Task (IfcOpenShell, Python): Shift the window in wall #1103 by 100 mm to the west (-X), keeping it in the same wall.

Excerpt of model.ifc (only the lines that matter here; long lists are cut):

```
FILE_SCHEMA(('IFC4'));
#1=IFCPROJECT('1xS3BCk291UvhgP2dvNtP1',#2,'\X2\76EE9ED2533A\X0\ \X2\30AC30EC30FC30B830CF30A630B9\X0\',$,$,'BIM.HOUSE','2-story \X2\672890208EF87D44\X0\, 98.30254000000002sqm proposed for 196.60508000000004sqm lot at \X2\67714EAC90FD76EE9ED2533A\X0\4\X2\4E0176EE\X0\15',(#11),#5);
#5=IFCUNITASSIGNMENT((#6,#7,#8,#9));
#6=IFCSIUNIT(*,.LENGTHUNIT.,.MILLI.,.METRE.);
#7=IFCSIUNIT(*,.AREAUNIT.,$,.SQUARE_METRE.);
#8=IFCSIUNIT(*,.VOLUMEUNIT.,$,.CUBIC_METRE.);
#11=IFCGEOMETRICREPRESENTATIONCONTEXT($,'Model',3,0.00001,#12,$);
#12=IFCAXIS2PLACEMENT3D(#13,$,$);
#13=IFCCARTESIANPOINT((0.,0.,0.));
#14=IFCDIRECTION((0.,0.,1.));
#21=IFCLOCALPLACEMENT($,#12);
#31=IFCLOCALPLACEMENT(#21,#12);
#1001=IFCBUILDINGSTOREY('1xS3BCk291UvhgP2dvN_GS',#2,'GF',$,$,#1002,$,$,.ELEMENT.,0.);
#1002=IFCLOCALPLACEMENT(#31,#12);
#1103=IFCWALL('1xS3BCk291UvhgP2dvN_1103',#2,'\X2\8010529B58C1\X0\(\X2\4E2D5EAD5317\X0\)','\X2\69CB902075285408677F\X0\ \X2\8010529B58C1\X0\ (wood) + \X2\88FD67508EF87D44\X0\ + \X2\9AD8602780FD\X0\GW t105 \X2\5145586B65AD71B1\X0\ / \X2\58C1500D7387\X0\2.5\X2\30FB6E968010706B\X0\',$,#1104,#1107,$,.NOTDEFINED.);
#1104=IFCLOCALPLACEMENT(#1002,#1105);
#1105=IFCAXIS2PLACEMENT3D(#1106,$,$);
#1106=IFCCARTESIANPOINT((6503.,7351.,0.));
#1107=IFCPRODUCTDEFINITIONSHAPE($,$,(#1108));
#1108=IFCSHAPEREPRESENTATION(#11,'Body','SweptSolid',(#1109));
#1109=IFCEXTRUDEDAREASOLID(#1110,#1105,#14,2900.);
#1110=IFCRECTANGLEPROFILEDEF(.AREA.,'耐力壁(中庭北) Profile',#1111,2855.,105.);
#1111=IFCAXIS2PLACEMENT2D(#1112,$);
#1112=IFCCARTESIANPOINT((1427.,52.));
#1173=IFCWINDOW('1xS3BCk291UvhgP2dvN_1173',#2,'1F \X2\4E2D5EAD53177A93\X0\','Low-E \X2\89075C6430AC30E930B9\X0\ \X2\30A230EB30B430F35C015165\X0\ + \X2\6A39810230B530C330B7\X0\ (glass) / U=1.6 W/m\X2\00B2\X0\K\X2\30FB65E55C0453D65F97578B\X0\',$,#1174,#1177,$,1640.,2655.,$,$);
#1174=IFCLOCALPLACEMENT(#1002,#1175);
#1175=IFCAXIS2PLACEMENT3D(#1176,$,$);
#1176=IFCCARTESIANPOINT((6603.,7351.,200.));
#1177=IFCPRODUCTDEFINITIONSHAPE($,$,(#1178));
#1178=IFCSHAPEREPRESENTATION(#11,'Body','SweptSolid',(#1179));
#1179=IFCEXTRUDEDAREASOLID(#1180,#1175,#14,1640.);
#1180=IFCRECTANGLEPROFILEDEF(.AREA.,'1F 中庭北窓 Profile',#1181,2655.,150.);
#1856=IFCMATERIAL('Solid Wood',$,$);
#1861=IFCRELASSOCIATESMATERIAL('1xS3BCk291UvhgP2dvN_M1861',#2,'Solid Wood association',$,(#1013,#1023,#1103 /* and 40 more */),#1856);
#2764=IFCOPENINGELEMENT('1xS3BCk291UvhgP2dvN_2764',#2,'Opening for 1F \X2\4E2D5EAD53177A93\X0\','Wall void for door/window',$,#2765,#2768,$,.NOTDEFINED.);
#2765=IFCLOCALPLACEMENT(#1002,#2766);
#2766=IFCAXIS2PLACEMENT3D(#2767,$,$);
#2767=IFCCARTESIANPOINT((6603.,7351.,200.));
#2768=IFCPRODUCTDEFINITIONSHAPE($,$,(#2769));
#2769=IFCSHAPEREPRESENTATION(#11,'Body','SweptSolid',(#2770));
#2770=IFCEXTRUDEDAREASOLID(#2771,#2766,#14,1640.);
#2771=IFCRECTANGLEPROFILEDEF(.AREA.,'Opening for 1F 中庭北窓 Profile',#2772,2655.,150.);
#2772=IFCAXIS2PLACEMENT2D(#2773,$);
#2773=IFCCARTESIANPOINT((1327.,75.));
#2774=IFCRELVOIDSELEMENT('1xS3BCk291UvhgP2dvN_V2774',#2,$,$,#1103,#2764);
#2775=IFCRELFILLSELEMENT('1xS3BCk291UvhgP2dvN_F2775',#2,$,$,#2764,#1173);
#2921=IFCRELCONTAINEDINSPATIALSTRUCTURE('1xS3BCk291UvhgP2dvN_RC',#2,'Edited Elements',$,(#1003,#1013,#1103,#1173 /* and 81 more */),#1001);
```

```python
import ifcopenshell
import ifcopenshell.api.geometry
import ifcopenshell.util.placement

model = ifcopenshell.open("model.ifc")

window = model.by_guid("1xS3BCk291UvhgP2dvN_1173")
opening = window.FillsVoids[0].RelatingOpeningElement
wall = opening.VoidsElements[0].RelatingBuildingElement

wall_matrix = ifcopenshell.util.placement.get_local_placement(wall.ObjectPlacement)
shift = wall_matrix[:3, 0] * -100.0
before = ifcopenshell.util.placement.get_local_placement(window.ObjectPlacement)[:3, 3].copy()

# The window is not placed relative to its opening, so move both.
for product in (opening, window):
    matrix = ifcopenshell.util.placement.get_local_placement(product.ObjectPlacement)
    matrix[:3, 3] += shift
    ifcopenshell.api.geometry.edit_object_placement(model, product=product, matrix=matrix, is_si=False)

after = ifcopenshell.util.placement.get_local_placement(window.ObjectPlacement)[:3, 3]
print("window moved by", (after - before).round(3) + 0.0)

model.write("model_edited.ifc")
```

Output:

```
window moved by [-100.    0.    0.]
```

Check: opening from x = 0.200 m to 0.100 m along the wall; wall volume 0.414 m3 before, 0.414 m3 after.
